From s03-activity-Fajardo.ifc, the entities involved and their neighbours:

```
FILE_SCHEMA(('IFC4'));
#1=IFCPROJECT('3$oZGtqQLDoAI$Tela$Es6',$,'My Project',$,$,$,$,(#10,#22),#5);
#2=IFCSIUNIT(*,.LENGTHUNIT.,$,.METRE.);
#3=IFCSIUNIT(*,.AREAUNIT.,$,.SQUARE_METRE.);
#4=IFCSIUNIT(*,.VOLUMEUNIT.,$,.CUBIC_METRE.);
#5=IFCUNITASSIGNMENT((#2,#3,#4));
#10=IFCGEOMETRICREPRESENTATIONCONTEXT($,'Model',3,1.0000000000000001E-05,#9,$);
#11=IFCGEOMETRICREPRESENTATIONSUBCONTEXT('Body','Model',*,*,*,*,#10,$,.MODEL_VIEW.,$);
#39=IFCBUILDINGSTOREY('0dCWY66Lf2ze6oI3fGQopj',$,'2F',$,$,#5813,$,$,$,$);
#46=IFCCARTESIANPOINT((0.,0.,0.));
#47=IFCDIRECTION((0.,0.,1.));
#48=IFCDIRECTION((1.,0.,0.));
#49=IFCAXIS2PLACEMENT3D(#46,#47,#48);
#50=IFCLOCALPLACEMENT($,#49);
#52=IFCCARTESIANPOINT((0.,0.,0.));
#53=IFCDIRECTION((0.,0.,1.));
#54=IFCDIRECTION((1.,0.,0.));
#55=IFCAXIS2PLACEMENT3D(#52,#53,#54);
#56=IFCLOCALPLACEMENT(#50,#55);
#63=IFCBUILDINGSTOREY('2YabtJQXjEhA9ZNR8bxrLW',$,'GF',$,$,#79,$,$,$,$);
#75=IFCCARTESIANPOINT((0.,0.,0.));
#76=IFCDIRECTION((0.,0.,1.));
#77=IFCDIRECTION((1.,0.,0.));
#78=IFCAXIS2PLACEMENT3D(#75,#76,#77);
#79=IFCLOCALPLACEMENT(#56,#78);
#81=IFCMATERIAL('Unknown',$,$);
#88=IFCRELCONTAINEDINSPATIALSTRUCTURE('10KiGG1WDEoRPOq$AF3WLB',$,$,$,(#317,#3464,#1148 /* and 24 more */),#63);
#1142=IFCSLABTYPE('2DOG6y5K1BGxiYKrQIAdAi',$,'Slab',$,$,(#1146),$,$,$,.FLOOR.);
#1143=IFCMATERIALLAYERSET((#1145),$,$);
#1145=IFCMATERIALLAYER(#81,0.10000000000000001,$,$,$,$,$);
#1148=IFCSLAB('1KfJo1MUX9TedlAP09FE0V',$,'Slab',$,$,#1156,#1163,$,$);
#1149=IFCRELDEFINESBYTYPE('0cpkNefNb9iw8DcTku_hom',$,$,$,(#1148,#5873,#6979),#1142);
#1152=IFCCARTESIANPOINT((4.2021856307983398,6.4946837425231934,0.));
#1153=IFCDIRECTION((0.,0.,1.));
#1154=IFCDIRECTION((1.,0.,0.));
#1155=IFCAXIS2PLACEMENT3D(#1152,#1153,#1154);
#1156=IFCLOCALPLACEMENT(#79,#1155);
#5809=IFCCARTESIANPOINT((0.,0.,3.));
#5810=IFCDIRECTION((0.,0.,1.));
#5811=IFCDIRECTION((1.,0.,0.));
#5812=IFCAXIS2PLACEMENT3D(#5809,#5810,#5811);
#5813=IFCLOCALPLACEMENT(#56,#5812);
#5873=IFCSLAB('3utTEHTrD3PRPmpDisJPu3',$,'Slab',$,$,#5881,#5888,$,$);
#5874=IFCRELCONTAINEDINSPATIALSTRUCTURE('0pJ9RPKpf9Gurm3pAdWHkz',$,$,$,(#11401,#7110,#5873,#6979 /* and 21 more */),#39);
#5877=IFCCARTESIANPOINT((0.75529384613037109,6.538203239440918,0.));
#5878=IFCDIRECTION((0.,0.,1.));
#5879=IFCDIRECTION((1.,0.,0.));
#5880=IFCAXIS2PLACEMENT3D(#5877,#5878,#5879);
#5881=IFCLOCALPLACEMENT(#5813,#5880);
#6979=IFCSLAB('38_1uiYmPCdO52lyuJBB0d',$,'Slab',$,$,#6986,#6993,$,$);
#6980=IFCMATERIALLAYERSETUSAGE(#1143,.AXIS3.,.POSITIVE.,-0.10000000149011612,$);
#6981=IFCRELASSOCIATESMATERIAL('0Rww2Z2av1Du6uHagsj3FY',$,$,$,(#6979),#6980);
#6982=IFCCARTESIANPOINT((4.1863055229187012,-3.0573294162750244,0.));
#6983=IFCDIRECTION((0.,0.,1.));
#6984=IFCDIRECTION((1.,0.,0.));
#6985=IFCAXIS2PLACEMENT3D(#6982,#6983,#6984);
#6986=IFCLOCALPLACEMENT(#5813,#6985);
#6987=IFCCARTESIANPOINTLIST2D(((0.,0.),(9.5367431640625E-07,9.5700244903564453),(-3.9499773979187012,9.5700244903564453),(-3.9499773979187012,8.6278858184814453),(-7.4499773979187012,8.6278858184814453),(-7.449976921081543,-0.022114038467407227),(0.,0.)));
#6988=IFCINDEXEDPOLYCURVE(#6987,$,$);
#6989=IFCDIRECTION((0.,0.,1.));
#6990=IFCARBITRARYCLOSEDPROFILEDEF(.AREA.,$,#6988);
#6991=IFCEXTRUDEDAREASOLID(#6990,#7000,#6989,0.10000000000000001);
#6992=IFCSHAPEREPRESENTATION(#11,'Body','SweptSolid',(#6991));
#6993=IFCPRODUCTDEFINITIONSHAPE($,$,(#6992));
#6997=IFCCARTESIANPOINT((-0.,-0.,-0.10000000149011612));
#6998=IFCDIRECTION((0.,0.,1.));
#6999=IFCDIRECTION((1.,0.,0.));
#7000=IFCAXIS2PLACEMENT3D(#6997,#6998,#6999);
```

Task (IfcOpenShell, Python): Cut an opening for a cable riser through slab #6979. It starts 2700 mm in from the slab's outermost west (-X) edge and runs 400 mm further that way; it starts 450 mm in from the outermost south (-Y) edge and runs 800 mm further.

```python
import numpy as np
import ifcopenshell
import ifcopenshell.api.feature
import ifcopenshell.api.geometry
import ifcopenshell.api.root
import ifcopenshell.geom
import ifcopenshell.util.placement
import ifcopenshell.util.representation
import ifcopenshell.util.shape
import ifcopenshell.util.unit

model = ifcopenshell.open("s03-activity-Fajardo.ifc")
unit_scale = ifcopenshell.util.unit.calculate_unit_scale(model)
settings = ifcopenshell.geom.settings()


def volume(element):
    """Net volume in cubic metres, openings subtracted."""
    shape = ifcopenshell.geom.create_shape(settings, element)
    return ifcopenshell.util.shape.get_volume(shape.geometry)


slab = model.by_guid("38_1uiYmPCdO52lyuJBB0d")
before = volume(slab)

# Extent in the slab's own axes, in metres. The edges named are its -X and -Y sides.
slab_shape = ifcopenshell.geom.create_shape(settings, slab)
vertices = ifcopenshell.util.shape.get_vertices(slab_shape.geometry)
x_min, y_min, bottom = vertices.min(axis=0)
top = vertices[:, 2].max()

opening = ifcopenshell.api.root.create_entity(model, ifc_class="IfcOpeningElement", name="Cable riser opening", predefined_type="OPENING")
context = ifcopenshell.util.representation.get_context(model, "Model", "Body", "MODEL_VIEW")
width, depth = 0.4, 0.8
outline = [(0.0, 0.0), (width, 0.0), (width, depth), (0.0, depth), (0.0, 0.0)]
# Overshoot both faces by 50 mm so the cut is clean.
shape = ifcopenshell.api.geometry.add_slab_representation(
    model, context=context, depth=top - bottom + 0.1, polyline=outline
)
ifcopenshell.api.geometry.assign_representation(model, product=opening, representation=shape)

matrix = ifcopenshell.util.placement.get_local_placement(slab.ObjectPlacement)
matrix[:, 3] = matrix @ np.append(np.array([x_min + 2.7, y_min + 0.45, bottom - 0.05]) / unit_scale, 1.0)
ifcopenshell.api.geometry.edit_object_placement(model, product=opening, matrix=matrix, is_si=False)
ifcopenshell.api.feature.add_feature(model, feature=opening, element=slab)

after = volume(slab)

print(f"slab volume {before:.3f} -> {after:.3f} m3")

model.write("s03-activity-Fajardo_v2.ifc")
```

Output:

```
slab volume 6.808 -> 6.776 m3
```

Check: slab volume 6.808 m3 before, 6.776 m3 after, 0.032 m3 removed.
